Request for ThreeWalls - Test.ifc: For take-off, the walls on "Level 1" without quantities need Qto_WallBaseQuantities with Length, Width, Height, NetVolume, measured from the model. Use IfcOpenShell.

First a look at what the model holds.

```python
import ifcopenshell
import ifcopenshell.util.element
import ifcopenshell.util.unit

model = ifcopenshell.open("ThreeWalls - Test.ifc")
print(model.schema)
for unit_type in ("LENGTHUNIT", "AREAUNIT", "VOLUMEUNIT"):
    print(unit_type, ifcopenshell.util.unit.calculate_unit_scale(model, unit_type))
storey = next(s for s in model.by_type("IfcBuildingStorey") if s.Name == "Level 1")
walls = [e for e in ifcopenshell.util.element.get_decomposition(storey) if e.is_a("IfcWall")]
for e in sorted(walls, key=lambda e: e.id()):
    print(e.id(), e.is_a(), e.Name, list(ifcopenshell.util.element.get_psets(e, qtos_only=True)), sep=" | ")
```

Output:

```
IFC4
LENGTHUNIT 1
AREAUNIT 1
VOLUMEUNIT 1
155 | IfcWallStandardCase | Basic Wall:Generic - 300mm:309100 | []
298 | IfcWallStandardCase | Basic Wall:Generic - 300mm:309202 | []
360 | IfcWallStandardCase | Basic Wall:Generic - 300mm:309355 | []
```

```python
import ifcopenshell
import ifcopenshell.api.pset
import ifcopenshell.geom
import ifcopenshell.util.element
import ifcopenshell.util.shape
import ifcopenshell.util.unit

model = ifcopenshell.open("ThreeWalls - Test.ifc")
unit_scale = ifcopenshell.util.unit.calculate_unit_scale(model)
volume_scale = ifcopenshell.util.unit.calculate_unit_scale(model, "VOLUMEUNIT")
settings = ifcopenshell.geom.settings()

storey = next(s for s in model.by_type("IfcBuildingStorey") if s.Name == "Level 1")
walls = [e for e in ifcopenshell.util.element.get_decomposition(storey) if e.is_a("IfcWall")]

for e in sorted(walls, key=lambda e: e.id()):
    if ifcopenshell.util.element.get_psets(e, qtos_only=True, should_inherit=False):
        continue
    # Geometry comes back in metres, in the element's own axes.
    shape = ifcopenshell.geom.create_shape(settings, e)
    values = {
        "Length": ifcopenshell.util.shape.get_x(shape.geometry) / unit_scale,
        "Width": ifcopenshell.util.shape.get_y(shape.geometry) / unit_scale,
        "Height": ifcopenshell.util.shape.get_z(shape.geometry) / unit_scale,
        "NetVolume": ifcopenshell.util.shape.get_volume(shape.geometry) / volume_scale,
    }
    qto = ifcopenshell.api.pset.add_qto(model, product=e, name="Qto_WallBaseQuantities")
    ifcopenshell.api.pset.edit_qto(model, qto=qto, properties=values)
    print(e.id(), {k: round(v, 3) for k, v in values.items()})

model.write("ThreeWalls - Test_v2.ifc")
```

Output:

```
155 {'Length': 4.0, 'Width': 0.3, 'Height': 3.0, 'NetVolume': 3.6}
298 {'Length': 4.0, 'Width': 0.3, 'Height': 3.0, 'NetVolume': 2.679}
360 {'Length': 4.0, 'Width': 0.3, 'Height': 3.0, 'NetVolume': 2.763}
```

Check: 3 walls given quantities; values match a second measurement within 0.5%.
